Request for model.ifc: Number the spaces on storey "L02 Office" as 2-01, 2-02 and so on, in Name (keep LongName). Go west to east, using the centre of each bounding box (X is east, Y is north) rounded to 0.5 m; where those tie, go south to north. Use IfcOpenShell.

First a look at what the model holds.

```python
import ifcopenshell
import ifcopenshell.util.element
import ifcopenshell.util.placement

model = ifcopenshell.open("model.ifc")
print(model.schema)
storey = next(s for s in model.by_type("IfcBuildingStorey") if s.Name == "L02 Office")
spaces = [e for e in ifcopenshell.util.element.get_decomposition(storey) if e.is_a("IfcSpace")]
for e in sorted(spaces, key=lambda e: e.id()):
    origin = ifcopenshell.util.placement.get_local_placement(e.ObjectPlacement)[:3, 3]
    print(e.id(), e.Name, e.LongName, origin.round(2) + 0.0, sep=" | ")
```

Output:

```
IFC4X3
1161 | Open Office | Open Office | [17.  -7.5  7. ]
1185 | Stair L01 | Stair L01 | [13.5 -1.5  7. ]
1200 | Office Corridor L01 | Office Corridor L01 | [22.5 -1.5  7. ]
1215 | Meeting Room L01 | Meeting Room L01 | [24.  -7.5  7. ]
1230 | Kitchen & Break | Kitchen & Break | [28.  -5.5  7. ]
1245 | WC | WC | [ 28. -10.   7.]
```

```python
import ifcopenshell
import ifcopenshell.geom
import ifcopenshell.util.element
import ifcopenshell.util.shape

model = ifcopenshell.open("model.ifc")
settings = ifcopenshell.geom.settings()
settings.set("use-world-coords", True)


def centre(element):
    shape = ifcopenshell.geom.create_shape(settings, element)
    return ifcopenshell.util.shape.get_bbox_centroid(shape.geometry)


storey = next(s for s in model.by_type("IfcBuildingStorey") if s.Name == "L02 Office")
spaces = [e for e in ifcopenshell.util.element.get_decomposition(storey) if e.is_a("IfcSpace")]

# Insertion points can sit at a corner or the storey origin, so sort by the geometry (in metres).
centres = {e: centre(e) for e in spaces}
spaces.sort(key=lambda e: (round(centres[e][0] / 0.5), centres[e][1]))

for i, e in enumerate(spaces, start=1):
    number = f"2-{i:02d}"
    e.Name = number
    print(e.id(), number)

model.write("model-out.ifc")
```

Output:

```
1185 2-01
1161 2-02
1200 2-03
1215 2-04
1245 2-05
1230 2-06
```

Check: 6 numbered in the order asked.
